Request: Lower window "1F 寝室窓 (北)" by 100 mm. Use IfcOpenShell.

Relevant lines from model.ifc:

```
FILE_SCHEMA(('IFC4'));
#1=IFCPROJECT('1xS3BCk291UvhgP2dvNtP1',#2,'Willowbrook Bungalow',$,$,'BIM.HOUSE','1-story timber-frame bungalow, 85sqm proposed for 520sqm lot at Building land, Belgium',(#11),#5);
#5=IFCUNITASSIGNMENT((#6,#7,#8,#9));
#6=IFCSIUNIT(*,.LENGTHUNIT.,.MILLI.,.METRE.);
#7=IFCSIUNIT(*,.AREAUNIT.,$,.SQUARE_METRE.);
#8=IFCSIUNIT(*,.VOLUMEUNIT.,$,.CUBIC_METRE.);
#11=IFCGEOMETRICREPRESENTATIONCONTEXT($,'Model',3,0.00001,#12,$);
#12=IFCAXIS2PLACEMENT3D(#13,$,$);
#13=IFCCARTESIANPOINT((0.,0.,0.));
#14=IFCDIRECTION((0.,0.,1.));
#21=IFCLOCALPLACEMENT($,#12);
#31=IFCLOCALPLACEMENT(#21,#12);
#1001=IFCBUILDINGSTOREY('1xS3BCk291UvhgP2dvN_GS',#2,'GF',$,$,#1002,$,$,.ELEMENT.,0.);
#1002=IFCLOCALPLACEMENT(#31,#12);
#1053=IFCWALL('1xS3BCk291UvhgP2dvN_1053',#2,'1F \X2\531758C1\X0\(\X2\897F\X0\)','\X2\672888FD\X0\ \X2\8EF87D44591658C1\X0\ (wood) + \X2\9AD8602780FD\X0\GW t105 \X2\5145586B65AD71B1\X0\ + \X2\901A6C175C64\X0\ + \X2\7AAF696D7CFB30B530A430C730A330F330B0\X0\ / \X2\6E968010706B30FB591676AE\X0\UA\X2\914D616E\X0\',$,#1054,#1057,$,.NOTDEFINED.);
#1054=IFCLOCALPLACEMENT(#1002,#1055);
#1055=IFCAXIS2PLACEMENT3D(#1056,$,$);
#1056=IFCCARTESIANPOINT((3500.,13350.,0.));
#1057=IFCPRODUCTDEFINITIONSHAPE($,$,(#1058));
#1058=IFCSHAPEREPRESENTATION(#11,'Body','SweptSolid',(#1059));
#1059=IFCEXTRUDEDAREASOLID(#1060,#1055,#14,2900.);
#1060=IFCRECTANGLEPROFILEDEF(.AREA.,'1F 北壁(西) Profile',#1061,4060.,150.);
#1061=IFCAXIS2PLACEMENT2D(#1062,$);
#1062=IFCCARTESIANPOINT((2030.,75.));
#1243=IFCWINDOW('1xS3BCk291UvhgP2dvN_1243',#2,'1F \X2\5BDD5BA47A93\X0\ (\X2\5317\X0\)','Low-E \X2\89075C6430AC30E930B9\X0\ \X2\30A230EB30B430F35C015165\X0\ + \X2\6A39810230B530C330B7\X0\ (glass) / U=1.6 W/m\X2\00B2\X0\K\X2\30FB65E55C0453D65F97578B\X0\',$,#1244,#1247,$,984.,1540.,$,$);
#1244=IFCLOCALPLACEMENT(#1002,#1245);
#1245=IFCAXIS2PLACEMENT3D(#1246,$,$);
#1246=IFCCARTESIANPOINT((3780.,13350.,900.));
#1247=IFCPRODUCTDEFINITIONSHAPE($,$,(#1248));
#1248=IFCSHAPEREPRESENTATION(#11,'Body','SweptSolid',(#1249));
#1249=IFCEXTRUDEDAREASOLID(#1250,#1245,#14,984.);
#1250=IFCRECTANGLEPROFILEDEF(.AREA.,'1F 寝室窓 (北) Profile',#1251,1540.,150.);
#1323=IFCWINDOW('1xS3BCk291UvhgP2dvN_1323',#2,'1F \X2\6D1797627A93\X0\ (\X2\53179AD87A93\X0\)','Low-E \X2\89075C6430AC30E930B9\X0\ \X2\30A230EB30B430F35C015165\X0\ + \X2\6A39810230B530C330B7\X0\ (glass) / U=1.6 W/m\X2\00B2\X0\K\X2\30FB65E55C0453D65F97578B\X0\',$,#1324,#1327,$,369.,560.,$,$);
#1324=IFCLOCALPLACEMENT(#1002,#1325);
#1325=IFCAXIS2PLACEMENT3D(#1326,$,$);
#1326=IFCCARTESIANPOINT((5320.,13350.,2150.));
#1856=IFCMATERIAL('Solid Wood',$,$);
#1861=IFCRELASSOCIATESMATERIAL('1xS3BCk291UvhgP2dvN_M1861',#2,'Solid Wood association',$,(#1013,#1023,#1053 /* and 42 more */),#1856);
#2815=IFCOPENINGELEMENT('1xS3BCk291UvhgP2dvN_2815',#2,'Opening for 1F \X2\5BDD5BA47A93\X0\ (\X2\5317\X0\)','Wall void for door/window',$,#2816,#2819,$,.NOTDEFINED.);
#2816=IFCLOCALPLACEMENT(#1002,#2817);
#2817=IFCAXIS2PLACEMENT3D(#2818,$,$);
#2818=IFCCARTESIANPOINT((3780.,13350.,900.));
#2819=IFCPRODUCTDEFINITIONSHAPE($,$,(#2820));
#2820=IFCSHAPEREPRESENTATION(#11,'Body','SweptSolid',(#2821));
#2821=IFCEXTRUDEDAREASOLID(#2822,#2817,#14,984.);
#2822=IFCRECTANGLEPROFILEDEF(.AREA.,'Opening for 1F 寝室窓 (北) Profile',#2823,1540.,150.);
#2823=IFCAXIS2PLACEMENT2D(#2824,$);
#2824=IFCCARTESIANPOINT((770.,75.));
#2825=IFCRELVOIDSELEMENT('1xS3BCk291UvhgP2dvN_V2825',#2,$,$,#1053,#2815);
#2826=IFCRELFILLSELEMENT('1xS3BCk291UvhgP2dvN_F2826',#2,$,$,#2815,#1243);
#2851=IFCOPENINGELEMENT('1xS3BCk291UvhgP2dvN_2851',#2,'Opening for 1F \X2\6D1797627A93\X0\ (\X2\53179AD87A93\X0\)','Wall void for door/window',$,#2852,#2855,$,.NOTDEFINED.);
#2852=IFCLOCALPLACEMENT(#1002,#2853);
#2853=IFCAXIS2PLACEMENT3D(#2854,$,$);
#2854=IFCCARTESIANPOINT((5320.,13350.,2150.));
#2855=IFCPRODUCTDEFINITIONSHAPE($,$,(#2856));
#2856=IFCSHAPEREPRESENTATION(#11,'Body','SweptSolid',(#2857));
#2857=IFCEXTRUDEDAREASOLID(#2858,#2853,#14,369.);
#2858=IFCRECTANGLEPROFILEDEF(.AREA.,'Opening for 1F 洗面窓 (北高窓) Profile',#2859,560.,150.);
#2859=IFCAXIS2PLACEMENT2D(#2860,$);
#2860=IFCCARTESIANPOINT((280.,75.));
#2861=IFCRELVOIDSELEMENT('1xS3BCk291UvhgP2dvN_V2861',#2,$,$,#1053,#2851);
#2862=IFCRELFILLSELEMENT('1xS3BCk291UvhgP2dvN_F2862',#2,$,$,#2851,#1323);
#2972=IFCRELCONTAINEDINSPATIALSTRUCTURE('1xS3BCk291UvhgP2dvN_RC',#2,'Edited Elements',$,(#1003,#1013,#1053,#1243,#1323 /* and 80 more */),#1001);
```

```python
import numpy as np
import ifcopenshell
import ifcopenshell.api.geometry
import ifcopenshell.util.placement
import ifcopenshell.util.unit

model = ifcopenshell.open("model.ifc")
unit_scale = ifcopenshell.util.unit.calculate_unit_scale(model)

window = model.by_guid("1xS3BCk291UvhgP2dvN_1243")
opening = window.FillsVoids[0].RelatingOpeningElement
dz = -0.1 / unit_scale

shift = np.array([0.0, 0.0, dz])
# The window is not placed relative to its opening, so move both.
for product in (opening, window):
    matrix = ifcopenshell.util.placement.get_local_placement(product.ObjectPlacement)
    matrix[:3, 3] += shift
    ifcopenshell.api.geometry.edit_object_placement(model, product=product, matrix=matrix, is_si=False)

print(f"moved by {dz * unit_scale:+.3f} m")

model.write("model_edited.ifc")
```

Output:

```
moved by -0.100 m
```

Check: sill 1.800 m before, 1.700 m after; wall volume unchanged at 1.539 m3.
